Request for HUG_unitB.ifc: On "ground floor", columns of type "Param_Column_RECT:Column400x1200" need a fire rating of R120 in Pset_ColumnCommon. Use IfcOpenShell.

First a look at what the model holds.

```python
import ifcopenshell
import ifcopenshell.util.element

model = ifcopenshell.open("HUG_unitB.ifc")
print(model.schema)
storey = next(s for s in model.by_type("IfcBuildingStorey") if s.Name == "ground floor")
columns = [e for e in ifcopenshell.util.element.get_decomposition(storey) if e.is_a("IfcColumn")]
seen = {}
for e in columns:
    element_type = ifcopenshell.util.element.get_type(e)
    key = (element_type.Name if element_type != e and element_type else None, ifcopenshell.util.element.get_pset(e, "Pset_ColumnCommon", "FireRating"))
    seen[key] = seen.get(key, 0) + 1
for (name, value), count in sorted(seen.items(), key=str):
    print(count, "x", name, "|", value)
```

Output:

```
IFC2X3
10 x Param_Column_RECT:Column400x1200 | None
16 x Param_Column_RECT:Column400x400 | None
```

```python
import ifcopenshell
import ifcopenshell.api.pset
import ifcopenshell.util.element

model = ifcopenshell.open("HUG_unitB.ifc")

storey = next(s for s in model.by_type("IfcBuildingStorey") if s.Name == "ground floor")
columns = [e for e in ifcopenshell.util.element.get_decomposition(storey) if e.is_a("IfcColumn")]

count = 0
for e in columns:
    element_type = ifcopenshell.util.element.get_type(e)
    if element_type in (None, e) or element_type.Name != "Param_Column_RECT:Column400x1200":
        continue
    # add_pset returns the element's existing set when there is one.
    pset = ifcopenshell.api.pset.add_pset(model, product=e, name="Pset_ColumnCommon")
    ifcopenshell.api.pset.edit_pset(model, pset=pset, properties={"FireRating": "R120"})
    count += 1

print(count, "columns updated")

model.write("HUG_unitB_updated.ifc")
```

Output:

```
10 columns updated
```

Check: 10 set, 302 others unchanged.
